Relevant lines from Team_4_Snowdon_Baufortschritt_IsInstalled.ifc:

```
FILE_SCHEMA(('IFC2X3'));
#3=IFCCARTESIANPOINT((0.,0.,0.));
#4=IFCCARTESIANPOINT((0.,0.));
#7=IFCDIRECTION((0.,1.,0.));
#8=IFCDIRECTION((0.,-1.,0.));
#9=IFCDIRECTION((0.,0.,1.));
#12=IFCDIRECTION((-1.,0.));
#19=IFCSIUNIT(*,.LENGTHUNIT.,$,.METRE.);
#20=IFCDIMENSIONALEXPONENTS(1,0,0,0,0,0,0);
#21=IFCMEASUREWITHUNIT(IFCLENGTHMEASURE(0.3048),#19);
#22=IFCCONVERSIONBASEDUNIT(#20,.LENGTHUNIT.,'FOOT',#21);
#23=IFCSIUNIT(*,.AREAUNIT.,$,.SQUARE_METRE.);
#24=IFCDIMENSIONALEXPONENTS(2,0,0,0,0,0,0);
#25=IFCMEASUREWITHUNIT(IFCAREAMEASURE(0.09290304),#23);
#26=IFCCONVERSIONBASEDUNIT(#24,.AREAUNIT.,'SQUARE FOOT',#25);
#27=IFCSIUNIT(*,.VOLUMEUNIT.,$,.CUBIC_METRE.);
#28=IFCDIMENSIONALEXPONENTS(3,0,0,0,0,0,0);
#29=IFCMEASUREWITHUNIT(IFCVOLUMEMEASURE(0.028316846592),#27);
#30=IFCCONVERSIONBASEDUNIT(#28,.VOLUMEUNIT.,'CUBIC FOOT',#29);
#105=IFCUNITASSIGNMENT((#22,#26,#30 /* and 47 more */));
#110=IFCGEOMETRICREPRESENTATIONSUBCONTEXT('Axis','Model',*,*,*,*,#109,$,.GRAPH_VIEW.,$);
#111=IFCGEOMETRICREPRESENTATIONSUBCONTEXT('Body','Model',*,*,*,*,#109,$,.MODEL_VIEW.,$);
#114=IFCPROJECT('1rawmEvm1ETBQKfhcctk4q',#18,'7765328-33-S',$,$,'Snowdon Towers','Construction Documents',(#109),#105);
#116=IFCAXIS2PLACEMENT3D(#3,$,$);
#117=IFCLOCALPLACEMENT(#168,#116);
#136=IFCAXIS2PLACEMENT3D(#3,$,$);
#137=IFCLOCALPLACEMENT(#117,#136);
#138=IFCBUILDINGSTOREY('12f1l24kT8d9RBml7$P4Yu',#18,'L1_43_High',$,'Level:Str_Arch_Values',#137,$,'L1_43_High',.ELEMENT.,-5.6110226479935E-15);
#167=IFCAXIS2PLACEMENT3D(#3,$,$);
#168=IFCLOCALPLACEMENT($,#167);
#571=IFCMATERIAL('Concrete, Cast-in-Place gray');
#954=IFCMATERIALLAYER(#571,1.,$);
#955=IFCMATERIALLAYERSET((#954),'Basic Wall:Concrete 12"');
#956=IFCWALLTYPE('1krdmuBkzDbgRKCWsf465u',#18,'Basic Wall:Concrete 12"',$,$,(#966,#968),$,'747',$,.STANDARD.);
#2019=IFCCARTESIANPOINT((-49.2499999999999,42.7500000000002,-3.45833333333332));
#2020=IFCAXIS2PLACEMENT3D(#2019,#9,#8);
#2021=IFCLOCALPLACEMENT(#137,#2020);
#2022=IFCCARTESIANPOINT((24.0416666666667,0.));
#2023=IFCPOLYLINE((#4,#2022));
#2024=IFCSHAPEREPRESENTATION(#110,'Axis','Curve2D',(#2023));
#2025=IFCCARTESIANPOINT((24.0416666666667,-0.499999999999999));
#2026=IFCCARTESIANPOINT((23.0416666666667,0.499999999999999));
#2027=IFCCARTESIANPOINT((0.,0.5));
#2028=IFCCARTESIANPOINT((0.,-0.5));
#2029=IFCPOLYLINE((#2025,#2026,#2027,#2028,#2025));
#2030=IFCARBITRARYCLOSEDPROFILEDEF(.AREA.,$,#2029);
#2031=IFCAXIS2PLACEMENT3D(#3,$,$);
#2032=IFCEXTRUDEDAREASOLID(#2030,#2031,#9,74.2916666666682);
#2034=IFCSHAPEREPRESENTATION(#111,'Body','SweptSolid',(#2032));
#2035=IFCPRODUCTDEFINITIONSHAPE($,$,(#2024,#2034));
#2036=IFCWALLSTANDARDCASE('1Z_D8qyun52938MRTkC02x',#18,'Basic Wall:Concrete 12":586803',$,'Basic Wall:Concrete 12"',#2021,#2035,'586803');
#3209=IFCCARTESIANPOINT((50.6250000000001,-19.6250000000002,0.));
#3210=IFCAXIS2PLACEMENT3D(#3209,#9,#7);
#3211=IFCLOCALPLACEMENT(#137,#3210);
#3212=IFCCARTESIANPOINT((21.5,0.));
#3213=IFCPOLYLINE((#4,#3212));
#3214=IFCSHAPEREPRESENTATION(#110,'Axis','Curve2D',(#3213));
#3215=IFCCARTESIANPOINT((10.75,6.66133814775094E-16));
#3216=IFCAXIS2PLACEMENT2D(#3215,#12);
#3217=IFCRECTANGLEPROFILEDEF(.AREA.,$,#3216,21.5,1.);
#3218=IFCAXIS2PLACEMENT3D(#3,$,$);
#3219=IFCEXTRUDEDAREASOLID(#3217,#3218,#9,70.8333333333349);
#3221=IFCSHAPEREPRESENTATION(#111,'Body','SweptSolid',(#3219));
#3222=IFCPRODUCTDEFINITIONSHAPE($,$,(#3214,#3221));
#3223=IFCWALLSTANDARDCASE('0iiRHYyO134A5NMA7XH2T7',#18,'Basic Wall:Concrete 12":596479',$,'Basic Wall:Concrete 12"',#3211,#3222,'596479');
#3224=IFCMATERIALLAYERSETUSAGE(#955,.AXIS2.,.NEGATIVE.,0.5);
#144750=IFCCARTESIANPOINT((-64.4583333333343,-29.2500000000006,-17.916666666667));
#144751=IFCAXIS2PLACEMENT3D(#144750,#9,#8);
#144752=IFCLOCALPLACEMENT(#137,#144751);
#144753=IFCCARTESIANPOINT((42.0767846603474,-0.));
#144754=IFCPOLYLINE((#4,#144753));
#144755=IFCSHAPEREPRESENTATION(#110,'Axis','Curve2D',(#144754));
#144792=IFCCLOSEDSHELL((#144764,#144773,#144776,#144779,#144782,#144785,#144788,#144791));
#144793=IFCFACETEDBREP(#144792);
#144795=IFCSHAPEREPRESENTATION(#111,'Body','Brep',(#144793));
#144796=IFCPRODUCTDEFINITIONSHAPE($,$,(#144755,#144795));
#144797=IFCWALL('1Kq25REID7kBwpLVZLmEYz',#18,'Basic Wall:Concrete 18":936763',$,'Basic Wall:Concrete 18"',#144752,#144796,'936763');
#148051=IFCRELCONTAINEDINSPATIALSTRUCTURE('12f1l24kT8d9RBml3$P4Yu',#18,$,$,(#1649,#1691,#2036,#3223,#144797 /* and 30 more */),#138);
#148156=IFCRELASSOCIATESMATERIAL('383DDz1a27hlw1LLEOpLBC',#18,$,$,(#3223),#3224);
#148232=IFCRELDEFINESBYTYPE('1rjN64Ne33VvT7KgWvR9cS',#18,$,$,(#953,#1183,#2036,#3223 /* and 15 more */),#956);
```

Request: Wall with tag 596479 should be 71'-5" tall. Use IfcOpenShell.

```python
import ifcopenshell
import ifcopenshell.geom
import ifcopenshell.util.representation
import ifcopenshell.util.shape
import ifcopenshell.util.unit

model = ifcopenshell.open("Team_4_Snowdon_Baufortschritt_IsInstalled.ifc")
unit_scale = ifcopenshell.util.unit.calculate_unit_scale(model)
settings = ifcopenshell.geom.settings()


def volume(element):
    """Net volume in cubic metres, openings subtracted."""
    shape = ifcopenshell.geom.create_shape(settings, element)
    return ifcopenshell.util.shape.get_volume(shape.geometry)


wall = model.by_id(3223)
before = volume(wall)

body = ifcopenshell.util.representation.get_representation(wall, "Model", "Body")
solid = body.Items[0]
old_height = solid.Depth
solid.Depth = 857 * 0.0254 / unit_scale
after = volume(wall)

print(f"height {old_height:g} -> {solid.Depth:g}, volume {before:.3f} -> {after:.3f} m3")

model.write("Team_4_Snowdon_Baufortschritt_IsInstalled_v2.ifc")
```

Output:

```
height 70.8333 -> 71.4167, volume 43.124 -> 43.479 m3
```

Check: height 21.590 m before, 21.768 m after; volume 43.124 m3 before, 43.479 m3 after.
